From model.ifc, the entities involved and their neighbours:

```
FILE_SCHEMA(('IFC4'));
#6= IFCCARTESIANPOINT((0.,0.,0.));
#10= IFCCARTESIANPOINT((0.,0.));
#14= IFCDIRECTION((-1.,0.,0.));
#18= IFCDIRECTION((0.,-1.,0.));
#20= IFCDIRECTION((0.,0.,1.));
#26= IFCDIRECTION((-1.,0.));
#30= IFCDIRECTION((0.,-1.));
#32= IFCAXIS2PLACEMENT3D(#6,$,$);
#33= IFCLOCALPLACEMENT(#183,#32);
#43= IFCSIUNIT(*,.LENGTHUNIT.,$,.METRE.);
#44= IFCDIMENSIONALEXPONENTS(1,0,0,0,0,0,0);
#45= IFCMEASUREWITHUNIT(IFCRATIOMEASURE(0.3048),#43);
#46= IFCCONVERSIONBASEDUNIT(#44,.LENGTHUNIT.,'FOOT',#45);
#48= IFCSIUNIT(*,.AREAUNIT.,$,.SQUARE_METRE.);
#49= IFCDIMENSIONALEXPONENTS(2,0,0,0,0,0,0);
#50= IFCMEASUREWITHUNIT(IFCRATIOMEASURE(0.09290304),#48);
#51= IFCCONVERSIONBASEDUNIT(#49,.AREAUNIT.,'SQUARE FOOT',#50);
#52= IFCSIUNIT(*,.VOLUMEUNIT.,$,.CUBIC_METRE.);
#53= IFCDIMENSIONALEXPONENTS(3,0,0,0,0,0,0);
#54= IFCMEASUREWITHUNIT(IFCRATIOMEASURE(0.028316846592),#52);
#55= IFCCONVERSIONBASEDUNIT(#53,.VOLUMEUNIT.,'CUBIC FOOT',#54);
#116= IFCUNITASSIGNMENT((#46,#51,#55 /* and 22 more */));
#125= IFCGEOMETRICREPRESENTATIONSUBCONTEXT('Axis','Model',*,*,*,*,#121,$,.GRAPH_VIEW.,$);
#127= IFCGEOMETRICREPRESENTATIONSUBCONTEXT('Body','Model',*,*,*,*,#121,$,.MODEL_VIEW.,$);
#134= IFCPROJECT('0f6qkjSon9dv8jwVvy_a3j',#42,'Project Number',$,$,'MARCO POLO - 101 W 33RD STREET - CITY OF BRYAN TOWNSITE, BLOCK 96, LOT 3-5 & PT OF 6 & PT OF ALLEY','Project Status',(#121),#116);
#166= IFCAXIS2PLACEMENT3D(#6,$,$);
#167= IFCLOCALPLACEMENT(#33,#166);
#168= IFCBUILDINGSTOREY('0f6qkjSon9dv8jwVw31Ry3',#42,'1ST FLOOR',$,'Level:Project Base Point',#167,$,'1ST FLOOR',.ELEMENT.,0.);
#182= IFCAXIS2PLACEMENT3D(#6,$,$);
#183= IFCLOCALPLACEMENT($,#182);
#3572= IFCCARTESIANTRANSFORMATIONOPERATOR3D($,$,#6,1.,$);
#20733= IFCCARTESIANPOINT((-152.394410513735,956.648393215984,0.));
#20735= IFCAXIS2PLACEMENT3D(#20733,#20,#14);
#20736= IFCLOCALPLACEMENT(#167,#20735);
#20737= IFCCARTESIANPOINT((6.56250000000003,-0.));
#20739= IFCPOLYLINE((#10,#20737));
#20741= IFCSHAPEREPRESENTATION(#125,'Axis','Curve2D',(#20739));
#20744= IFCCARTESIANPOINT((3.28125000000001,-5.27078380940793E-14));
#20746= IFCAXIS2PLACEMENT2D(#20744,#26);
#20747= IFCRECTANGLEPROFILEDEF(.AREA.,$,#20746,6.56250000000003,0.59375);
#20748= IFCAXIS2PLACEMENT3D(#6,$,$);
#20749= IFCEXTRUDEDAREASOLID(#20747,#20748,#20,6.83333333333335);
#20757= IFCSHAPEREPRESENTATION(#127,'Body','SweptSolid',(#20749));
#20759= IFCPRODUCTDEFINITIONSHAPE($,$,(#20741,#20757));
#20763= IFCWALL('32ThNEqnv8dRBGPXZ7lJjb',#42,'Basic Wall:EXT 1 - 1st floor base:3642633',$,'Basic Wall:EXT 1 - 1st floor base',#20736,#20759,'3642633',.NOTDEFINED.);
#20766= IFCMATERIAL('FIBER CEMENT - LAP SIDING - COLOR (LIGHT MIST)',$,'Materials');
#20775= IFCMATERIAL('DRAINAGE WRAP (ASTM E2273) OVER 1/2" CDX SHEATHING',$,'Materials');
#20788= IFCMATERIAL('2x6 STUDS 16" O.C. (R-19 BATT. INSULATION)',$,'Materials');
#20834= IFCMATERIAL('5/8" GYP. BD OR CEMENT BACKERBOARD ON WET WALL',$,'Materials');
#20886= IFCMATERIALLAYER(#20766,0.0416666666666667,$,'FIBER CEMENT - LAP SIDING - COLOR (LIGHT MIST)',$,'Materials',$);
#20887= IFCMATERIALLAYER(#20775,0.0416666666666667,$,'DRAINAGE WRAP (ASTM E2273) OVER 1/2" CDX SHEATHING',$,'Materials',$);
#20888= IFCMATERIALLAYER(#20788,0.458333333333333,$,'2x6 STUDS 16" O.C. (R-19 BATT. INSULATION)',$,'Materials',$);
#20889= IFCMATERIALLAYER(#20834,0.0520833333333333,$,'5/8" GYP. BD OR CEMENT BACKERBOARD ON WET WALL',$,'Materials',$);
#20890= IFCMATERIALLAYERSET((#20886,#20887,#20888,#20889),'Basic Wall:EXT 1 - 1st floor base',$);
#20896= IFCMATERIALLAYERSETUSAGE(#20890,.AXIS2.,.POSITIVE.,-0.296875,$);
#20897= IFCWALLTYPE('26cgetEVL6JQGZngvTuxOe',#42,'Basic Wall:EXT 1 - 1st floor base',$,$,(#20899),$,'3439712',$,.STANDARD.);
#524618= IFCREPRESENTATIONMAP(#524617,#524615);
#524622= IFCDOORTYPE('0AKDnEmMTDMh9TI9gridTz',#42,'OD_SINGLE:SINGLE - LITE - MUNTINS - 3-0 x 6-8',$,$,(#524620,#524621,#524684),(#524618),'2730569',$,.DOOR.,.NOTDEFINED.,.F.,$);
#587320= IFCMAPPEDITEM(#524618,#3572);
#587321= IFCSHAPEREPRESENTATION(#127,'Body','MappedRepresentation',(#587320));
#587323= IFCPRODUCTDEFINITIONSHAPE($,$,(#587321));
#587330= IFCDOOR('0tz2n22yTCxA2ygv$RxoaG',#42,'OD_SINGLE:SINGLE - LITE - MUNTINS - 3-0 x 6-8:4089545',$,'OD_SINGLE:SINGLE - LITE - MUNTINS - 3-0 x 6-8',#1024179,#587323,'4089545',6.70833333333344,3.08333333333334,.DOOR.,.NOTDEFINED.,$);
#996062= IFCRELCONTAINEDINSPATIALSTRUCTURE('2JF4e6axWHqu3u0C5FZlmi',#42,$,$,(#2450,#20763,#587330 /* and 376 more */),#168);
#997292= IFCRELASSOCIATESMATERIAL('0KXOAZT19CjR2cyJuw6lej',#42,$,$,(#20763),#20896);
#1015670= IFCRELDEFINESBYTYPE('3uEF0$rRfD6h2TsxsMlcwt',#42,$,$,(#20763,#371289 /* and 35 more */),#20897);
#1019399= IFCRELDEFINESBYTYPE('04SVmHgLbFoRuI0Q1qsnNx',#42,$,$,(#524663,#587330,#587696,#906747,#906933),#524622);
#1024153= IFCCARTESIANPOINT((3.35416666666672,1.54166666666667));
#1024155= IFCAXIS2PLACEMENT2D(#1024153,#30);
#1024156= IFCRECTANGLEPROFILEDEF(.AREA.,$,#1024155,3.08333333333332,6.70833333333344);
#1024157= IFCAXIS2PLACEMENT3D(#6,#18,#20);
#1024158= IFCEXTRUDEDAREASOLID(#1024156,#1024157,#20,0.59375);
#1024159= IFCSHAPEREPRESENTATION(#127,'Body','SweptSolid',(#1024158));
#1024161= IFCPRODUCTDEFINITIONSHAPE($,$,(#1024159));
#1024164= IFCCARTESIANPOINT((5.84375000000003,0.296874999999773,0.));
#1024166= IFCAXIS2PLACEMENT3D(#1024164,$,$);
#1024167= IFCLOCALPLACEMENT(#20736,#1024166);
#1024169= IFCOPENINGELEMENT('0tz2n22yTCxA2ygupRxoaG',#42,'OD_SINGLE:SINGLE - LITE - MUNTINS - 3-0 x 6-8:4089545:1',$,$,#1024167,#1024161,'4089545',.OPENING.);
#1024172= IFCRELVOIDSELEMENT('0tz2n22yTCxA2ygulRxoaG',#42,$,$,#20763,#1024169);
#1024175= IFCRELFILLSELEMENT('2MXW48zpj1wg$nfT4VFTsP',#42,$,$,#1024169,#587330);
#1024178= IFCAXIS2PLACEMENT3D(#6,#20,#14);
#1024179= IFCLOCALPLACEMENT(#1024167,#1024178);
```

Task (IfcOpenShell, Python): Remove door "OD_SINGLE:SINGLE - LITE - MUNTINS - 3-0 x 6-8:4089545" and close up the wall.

```python
import ifcopenshell
import ifcopenshell.api.feature
import ifcopenshell.api.root
import ifcopenshell.geom
import ifcopenshell.util.shape

model = ifcopenshell.open("model.ifc")
settings = ifcopenshell.geom.settings()


def volume(element):
    """Net volume in cubic metres, openings subtracted."""
    shape = ifcopenshell.geom.create_shape(settings, element)
    return ifcopenshell.util.shape.get_volume(shape.geometry)


door = model.by_guid("0tz2n22yTCxA2ygv$RxoaG")
opening = door.FillsVoids[0].RelatingOpeningElement
wall = opening.VoidsElements[0].RelatingBuildingElement
before = volume(wall)

ifcopenshell.api.root.remove_product(model, product=door)
ifcopenshell.api.feature.remove_feature(model, feature=opening)

after = volume(wall)

print(f"wall volume {before:.3f} -> {after:.3f} m3")

model.write("model_edited.ifc")
```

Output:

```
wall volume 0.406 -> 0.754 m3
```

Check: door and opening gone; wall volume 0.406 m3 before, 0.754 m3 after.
